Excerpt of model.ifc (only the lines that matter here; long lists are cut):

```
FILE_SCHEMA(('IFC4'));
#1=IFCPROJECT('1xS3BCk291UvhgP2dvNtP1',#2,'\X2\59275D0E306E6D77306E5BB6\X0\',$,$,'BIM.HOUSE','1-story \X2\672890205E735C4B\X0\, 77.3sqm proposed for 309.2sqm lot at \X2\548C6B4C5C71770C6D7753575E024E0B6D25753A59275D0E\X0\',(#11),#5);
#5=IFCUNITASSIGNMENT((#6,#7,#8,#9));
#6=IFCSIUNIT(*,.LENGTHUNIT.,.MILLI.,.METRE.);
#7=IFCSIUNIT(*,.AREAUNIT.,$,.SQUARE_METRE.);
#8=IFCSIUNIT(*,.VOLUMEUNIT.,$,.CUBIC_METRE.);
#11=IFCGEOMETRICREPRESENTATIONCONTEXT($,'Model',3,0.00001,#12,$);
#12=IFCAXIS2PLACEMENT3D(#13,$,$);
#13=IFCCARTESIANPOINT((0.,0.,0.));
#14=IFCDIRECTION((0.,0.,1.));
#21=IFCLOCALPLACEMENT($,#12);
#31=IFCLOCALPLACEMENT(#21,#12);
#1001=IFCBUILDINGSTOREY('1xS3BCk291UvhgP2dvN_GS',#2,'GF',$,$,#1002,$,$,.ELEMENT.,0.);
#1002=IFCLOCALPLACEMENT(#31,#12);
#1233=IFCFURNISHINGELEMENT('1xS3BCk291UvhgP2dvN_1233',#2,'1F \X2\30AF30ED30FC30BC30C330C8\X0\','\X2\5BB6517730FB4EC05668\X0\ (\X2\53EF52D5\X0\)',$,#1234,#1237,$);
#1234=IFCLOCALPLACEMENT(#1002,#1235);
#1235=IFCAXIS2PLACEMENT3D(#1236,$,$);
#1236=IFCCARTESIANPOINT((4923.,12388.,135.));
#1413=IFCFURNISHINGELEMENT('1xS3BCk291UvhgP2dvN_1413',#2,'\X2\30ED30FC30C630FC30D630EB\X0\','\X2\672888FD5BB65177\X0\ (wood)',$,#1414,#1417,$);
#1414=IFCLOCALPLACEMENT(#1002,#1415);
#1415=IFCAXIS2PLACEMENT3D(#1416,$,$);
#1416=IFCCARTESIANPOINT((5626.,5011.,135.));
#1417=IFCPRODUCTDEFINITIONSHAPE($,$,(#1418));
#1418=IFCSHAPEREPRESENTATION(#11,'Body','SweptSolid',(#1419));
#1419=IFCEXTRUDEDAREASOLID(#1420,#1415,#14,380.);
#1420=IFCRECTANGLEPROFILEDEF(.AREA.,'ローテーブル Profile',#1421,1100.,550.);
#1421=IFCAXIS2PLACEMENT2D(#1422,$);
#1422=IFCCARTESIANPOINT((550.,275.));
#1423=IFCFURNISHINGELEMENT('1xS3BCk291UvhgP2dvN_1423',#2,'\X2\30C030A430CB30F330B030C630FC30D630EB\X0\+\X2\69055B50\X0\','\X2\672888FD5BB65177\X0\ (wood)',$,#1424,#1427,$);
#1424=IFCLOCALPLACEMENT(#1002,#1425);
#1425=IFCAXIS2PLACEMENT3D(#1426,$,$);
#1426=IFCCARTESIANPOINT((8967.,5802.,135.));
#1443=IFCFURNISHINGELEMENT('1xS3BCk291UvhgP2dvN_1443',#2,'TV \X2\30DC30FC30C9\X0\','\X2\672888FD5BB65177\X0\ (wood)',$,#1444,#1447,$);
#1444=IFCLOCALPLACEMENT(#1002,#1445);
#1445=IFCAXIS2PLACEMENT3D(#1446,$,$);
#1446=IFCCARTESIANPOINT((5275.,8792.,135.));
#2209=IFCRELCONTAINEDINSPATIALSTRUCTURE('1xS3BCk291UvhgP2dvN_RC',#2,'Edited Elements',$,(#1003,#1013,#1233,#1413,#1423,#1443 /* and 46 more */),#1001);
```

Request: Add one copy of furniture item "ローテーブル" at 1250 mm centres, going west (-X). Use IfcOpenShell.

```python
import numpy as np
import ifcopenshell
import ifcopenshell.api.geometry
import ifcopenshell.api.root
import ifcopenshell.util.element
import ifcopenshell.util.placement

model = ifcopenshell.open("model.ifc")


def reuse_history(source, copy):
    """copy_class also copies each property set's owner history, people and application; keep the originals."""
    for rel in copy.IsDefinedBy:
        if rel.is_a("IfcRelDefinesByProperties") and (history := rel.RelatingPropertyDefinition.OwnerHistory):
            rel.RelatingPropertyDefinition.OwnerHistory = source.OwnerHistory
            ifcopenshell.util.element.remove_deep2(model, history)


source = model.by_id(1413)
base = ifcopenshell.util.placement.get_local_placement(source.ObjectPlacement)
step = np.array([-1.0, 0.0, 0.0]) * 1250.0

for i in range(1, 2):
    copy = ifcopenshell.api.root.copy_class(model, product=source)
    copy.Representation = ifcopenshell.util.element.copy_deep(
        model, source.Representation, exclude=["IfcGeometricRepresentationContext", "IfcRepresentationMap"]
    )
    reuse_history(source, copy)
    matrix = base.copy()
    matrix[:3, 3] += i * step
    print("added at", matrix[:3, 3].round(3) + 0.0)
    ifcopenshell.api.geometry.edit_object_placement(model, product=copy, matrix=matrix, is_si=False)

model.write("model_v2.ifc")
```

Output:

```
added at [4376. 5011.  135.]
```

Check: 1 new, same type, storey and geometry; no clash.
